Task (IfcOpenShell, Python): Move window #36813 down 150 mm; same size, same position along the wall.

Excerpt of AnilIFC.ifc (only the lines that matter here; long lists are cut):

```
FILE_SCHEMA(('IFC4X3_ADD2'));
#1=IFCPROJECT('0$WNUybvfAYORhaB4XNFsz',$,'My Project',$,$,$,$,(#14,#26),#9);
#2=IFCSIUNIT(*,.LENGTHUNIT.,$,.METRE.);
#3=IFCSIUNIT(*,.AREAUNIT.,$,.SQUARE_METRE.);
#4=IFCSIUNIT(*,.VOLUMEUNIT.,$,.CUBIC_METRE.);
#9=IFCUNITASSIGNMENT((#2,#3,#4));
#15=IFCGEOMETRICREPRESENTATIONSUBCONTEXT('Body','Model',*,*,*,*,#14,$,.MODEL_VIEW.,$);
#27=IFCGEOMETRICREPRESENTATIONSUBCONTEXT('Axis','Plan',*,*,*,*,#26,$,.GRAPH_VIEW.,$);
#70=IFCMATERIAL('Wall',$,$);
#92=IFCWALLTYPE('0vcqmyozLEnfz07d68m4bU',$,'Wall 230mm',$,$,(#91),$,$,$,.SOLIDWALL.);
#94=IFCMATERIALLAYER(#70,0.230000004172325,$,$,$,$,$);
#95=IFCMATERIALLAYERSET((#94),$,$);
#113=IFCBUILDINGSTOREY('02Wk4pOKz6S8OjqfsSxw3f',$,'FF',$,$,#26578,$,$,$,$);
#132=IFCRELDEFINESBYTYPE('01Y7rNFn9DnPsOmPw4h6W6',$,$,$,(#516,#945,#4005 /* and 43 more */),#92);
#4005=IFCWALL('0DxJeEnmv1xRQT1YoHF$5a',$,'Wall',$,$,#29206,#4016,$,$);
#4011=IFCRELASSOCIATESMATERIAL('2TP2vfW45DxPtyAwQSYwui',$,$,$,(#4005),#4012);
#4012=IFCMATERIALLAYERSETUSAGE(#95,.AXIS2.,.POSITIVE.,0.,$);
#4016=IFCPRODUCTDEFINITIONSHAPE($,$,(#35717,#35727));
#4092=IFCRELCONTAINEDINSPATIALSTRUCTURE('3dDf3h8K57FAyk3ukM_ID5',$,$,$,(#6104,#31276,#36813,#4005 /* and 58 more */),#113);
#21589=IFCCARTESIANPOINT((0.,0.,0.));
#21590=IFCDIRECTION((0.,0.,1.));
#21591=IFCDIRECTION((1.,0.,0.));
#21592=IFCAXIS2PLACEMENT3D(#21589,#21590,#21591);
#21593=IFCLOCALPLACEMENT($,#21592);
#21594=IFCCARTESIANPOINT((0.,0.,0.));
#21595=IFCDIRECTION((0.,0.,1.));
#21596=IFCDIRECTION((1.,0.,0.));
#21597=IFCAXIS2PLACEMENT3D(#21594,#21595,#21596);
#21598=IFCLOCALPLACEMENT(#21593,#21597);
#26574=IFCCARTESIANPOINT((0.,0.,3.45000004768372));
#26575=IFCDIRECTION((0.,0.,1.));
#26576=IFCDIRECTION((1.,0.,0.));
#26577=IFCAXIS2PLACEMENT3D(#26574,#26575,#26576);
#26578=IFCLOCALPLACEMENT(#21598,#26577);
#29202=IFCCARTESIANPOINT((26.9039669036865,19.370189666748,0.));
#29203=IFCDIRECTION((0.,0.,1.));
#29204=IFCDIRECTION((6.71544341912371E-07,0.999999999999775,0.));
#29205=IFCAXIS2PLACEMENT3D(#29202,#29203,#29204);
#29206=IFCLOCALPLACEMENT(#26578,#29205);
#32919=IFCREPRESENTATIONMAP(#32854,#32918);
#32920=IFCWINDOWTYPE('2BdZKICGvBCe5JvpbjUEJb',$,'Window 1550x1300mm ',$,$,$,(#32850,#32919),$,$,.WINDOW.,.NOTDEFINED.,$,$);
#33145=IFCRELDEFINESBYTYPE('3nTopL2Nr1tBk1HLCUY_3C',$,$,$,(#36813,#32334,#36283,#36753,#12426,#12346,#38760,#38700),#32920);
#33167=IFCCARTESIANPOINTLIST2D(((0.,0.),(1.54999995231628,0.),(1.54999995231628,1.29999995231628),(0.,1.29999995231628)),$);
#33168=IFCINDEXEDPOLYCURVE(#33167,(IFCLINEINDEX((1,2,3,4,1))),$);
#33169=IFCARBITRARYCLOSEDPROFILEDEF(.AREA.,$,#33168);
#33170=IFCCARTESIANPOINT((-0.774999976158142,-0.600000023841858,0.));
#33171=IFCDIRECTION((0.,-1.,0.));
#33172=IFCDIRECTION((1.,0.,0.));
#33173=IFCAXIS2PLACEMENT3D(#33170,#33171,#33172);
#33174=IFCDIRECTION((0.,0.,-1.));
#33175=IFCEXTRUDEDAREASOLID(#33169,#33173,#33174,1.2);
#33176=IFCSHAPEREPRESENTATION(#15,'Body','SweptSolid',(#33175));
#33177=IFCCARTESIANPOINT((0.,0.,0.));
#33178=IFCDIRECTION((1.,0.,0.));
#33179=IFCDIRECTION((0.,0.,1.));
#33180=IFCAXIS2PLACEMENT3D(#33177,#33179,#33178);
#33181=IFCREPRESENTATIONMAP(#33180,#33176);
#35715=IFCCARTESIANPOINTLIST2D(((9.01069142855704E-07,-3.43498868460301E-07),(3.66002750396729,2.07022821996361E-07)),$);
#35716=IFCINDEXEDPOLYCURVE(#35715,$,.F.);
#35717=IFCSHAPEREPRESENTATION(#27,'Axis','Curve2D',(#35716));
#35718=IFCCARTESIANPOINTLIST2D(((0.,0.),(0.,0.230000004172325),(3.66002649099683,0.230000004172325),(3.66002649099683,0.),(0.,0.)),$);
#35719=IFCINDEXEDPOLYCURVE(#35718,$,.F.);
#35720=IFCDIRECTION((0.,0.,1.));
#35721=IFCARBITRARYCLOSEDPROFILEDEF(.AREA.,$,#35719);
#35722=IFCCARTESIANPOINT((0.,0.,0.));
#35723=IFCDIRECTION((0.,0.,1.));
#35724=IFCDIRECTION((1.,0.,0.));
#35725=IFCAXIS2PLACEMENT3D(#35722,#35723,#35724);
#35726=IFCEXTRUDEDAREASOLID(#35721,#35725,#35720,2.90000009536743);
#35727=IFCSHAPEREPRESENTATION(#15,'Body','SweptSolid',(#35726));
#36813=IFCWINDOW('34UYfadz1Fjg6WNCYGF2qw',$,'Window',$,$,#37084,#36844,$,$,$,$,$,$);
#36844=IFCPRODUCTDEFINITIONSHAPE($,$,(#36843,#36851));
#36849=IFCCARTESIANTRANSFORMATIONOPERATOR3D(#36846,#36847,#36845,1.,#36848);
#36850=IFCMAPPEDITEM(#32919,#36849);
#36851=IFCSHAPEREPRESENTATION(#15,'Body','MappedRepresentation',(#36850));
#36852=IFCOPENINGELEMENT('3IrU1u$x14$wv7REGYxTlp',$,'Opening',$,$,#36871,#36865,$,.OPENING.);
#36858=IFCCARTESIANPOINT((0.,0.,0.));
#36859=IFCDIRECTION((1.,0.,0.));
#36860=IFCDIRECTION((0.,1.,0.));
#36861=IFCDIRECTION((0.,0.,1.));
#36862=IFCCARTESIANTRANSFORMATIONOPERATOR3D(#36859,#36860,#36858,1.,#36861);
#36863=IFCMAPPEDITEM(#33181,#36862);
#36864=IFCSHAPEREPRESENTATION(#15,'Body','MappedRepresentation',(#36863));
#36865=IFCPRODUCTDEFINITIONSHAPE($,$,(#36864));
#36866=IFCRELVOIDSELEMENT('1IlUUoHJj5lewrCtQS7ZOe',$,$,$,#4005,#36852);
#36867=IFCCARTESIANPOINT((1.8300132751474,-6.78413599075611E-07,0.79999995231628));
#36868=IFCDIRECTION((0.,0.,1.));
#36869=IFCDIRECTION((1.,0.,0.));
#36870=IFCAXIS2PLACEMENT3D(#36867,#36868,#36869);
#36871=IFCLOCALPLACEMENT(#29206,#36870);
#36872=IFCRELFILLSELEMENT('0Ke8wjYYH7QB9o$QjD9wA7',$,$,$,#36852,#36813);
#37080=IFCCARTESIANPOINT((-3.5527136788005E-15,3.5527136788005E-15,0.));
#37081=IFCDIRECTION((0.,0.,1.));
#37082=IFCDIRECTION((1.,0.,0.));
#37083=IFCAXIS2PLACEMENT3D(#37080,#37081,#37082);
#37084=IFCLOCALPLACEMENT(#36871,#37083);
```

```python
import numpy as np
import ifcopenshell
import ifcopenshell.api.geometry
import ifcopenshell.util.placement
import ifcopenshell.util.unit

model = ifcopenshell.open("AnilIFC.ifc")
unit_scale = ifcopenshell.util.unit.calculate_unit_scale(model)

window = model.by_guid("34UYfadz1Fjg6WNCYGF2qw")
opening = window.FillsVoids[0].RelatingOpeningElement
dz = -0.15

shift = np.array([0.0, 0.0, dz])
# The window is placed relative to its opening, so it follows when the opening moves.
matrix = ifcopenshell.util.placement.get_local_placement(opening.ObjectPlacement)
matrix[:3, 3] += shift
ifcopenshell.api.geometry.edit_object_placement(
    model, product=opening, matrix=matrix, is_si=False, should_transform_children=True
)

print(f"moved by {dz * unit_scale:+.3f} m")

model.write("AnilIFC_rev.ifc")
```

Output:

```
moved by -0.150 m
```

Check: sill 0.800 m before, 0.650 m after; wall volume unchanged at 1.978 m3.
